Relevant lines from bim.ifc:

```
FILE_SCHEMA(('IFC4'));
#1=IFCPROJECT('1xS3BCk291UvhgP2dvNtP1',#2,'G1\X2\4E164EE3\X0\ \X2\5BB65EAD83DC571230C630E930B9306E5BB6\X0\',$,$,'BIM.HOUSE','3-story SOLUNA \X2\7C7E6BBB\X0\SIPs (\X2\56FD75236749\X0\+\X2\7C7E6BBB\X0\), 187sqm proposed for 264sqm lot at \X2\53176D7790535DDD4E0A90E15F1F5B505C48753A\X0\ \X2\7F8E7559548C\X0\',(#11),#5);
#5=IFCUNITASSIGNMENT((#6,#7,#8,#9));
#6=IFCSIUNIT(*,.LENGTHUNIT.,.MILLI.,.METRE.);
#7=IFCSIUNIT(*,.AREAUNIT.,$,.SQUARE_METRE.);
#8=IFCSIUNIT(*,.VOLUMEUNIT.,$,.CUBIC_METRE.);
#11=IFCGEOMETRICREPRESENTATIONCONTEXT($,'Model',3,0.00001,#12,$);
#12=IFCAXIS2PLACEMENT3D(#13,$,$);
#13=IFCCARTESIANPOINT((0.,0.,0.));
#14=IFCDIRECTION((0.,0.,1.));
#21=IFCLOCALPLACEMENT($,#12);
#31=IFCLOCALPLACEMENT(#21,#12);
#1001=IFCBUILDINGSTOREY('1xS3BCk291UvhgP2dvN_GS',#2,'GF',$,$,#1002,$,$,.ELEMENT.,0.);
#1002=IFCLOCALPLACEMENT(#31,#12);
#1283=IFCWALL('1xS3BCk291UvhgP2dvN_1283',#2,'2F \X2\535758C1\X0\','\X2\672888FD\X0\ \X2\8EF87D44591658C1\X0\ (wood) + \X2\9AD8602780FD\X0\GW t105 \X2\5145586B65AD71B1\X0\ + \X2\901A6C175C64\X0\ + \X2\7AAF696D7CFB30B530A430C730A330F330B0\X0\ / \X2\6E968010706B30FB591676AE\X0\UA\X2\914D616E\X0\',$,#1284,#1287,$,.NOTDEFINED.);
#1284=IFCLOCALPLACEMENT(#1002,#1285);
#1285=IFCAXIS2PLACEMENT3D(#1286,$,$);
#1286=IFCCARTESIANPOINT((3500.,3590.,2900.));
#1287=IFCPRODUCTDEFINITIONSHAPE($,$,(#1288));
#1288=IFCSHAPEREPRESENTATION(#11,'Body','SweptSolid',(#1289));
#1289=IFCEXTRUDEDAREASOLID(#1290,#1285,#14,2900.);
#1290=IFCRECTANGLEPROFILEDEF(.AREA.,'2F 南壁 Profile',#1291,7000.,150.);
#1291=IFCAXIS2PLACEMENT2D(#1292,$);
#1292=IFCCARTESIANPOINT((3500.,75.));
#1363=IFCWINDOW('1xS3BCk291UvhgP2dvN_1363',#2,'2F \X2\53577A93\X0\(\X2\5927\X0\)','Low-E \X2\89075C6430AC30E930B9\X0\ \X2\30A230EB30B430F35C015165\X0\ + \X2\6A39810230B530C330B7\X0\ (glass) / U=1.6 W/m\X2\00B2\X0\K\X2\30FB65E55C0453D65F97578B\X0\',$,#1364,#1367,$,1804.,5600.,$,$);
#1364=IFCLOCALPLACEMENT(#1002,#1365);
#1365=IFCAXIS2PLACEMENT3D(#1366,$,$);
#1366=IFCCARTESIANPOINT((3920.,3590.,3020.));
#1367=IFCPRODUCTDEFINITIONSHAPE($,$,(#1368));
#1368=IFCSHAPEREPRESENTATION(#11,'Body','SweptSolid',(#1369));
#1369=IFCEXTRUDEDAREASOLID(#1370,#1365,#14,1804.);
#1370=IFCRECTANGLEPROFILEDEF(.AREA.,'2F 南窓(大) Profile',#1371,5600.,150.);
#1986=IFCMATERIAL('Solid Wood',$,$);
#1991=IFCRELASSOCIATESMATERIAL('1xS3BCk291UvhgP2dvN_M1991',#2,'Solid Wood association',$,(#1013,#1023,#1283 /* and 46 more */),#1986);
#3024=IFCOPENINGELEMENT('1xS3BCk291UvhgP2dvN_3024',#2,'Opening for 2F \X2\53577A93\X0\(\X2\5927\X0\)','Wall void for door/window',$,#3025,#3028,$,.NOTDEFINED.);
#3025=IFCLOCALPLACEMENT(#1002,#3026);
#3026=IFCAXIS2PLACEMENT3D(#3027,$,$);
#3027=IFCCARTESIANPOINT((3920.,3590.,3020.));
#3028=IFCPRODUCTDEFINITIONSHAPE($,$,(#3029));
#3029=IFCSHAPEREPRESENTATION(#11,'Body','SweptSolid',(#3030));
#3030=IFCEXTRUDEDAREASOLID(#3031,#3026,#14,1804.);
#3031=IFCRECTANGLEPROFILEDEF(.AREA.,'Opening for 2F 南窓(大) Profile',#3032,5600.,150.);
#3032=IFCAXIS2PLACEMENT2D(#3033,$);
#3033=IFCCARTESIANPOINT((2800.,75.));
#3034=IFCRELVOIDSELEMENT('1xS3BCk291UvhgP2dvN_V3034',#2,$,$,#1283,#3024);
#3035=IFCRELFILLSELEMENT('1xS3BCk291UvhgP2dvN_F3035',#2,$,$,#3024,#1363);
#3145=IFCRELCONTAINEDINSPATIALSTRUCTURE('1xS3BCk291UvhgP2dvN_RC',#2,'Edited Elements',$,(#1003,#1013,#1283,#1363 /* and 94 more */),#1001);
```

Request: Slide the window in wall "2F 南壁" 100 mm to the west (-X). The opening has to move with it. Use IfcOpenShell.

```python
import ifcopenshell
import ifcopenshell.api.geometry
import ifcopenshell.util.placement

model = ifcopenshell.open("bim.ifc")

window = model.by_guid("1xS3BCk291UvhgP2dvN_1363")
opening = window.FillsVoids[0].RelatingOpeningElement
wall = opening.VoidsElements[0].RelatingBuildingElement

wall_matrix = ifcopenshell.util.placement.get_local_placement(wall.ObjectPlacement)
shift = wall_matrix[:3, 0] * -100.0
before = ifcopenshell.util.placement.get_local_placement(window.ObjectPlacement)[:3, 3].copy()

# The window is not placed relative to its opening, so move both.
for product in (opening, window):
    matrix = ifcopenshell.util.placement.get_local_placement(product.ObjectPlacement)
    matrix[:3, 3] += shift
    ifcopenshell.api.geometry.edit_object_placement(model, product=product, matrix=matrix, is_si=False)

after = ifcopenshell.util.placement.get_local_placement(window.ObjectPlacement)[:3, 3]
print("window moved by", (after - before).round(3) + 0.0)

model.write("bim_v2.ifc")
```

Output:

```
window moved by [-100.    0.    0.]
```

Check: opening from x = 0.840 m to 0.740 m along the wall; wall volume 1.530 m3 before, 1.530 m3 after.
